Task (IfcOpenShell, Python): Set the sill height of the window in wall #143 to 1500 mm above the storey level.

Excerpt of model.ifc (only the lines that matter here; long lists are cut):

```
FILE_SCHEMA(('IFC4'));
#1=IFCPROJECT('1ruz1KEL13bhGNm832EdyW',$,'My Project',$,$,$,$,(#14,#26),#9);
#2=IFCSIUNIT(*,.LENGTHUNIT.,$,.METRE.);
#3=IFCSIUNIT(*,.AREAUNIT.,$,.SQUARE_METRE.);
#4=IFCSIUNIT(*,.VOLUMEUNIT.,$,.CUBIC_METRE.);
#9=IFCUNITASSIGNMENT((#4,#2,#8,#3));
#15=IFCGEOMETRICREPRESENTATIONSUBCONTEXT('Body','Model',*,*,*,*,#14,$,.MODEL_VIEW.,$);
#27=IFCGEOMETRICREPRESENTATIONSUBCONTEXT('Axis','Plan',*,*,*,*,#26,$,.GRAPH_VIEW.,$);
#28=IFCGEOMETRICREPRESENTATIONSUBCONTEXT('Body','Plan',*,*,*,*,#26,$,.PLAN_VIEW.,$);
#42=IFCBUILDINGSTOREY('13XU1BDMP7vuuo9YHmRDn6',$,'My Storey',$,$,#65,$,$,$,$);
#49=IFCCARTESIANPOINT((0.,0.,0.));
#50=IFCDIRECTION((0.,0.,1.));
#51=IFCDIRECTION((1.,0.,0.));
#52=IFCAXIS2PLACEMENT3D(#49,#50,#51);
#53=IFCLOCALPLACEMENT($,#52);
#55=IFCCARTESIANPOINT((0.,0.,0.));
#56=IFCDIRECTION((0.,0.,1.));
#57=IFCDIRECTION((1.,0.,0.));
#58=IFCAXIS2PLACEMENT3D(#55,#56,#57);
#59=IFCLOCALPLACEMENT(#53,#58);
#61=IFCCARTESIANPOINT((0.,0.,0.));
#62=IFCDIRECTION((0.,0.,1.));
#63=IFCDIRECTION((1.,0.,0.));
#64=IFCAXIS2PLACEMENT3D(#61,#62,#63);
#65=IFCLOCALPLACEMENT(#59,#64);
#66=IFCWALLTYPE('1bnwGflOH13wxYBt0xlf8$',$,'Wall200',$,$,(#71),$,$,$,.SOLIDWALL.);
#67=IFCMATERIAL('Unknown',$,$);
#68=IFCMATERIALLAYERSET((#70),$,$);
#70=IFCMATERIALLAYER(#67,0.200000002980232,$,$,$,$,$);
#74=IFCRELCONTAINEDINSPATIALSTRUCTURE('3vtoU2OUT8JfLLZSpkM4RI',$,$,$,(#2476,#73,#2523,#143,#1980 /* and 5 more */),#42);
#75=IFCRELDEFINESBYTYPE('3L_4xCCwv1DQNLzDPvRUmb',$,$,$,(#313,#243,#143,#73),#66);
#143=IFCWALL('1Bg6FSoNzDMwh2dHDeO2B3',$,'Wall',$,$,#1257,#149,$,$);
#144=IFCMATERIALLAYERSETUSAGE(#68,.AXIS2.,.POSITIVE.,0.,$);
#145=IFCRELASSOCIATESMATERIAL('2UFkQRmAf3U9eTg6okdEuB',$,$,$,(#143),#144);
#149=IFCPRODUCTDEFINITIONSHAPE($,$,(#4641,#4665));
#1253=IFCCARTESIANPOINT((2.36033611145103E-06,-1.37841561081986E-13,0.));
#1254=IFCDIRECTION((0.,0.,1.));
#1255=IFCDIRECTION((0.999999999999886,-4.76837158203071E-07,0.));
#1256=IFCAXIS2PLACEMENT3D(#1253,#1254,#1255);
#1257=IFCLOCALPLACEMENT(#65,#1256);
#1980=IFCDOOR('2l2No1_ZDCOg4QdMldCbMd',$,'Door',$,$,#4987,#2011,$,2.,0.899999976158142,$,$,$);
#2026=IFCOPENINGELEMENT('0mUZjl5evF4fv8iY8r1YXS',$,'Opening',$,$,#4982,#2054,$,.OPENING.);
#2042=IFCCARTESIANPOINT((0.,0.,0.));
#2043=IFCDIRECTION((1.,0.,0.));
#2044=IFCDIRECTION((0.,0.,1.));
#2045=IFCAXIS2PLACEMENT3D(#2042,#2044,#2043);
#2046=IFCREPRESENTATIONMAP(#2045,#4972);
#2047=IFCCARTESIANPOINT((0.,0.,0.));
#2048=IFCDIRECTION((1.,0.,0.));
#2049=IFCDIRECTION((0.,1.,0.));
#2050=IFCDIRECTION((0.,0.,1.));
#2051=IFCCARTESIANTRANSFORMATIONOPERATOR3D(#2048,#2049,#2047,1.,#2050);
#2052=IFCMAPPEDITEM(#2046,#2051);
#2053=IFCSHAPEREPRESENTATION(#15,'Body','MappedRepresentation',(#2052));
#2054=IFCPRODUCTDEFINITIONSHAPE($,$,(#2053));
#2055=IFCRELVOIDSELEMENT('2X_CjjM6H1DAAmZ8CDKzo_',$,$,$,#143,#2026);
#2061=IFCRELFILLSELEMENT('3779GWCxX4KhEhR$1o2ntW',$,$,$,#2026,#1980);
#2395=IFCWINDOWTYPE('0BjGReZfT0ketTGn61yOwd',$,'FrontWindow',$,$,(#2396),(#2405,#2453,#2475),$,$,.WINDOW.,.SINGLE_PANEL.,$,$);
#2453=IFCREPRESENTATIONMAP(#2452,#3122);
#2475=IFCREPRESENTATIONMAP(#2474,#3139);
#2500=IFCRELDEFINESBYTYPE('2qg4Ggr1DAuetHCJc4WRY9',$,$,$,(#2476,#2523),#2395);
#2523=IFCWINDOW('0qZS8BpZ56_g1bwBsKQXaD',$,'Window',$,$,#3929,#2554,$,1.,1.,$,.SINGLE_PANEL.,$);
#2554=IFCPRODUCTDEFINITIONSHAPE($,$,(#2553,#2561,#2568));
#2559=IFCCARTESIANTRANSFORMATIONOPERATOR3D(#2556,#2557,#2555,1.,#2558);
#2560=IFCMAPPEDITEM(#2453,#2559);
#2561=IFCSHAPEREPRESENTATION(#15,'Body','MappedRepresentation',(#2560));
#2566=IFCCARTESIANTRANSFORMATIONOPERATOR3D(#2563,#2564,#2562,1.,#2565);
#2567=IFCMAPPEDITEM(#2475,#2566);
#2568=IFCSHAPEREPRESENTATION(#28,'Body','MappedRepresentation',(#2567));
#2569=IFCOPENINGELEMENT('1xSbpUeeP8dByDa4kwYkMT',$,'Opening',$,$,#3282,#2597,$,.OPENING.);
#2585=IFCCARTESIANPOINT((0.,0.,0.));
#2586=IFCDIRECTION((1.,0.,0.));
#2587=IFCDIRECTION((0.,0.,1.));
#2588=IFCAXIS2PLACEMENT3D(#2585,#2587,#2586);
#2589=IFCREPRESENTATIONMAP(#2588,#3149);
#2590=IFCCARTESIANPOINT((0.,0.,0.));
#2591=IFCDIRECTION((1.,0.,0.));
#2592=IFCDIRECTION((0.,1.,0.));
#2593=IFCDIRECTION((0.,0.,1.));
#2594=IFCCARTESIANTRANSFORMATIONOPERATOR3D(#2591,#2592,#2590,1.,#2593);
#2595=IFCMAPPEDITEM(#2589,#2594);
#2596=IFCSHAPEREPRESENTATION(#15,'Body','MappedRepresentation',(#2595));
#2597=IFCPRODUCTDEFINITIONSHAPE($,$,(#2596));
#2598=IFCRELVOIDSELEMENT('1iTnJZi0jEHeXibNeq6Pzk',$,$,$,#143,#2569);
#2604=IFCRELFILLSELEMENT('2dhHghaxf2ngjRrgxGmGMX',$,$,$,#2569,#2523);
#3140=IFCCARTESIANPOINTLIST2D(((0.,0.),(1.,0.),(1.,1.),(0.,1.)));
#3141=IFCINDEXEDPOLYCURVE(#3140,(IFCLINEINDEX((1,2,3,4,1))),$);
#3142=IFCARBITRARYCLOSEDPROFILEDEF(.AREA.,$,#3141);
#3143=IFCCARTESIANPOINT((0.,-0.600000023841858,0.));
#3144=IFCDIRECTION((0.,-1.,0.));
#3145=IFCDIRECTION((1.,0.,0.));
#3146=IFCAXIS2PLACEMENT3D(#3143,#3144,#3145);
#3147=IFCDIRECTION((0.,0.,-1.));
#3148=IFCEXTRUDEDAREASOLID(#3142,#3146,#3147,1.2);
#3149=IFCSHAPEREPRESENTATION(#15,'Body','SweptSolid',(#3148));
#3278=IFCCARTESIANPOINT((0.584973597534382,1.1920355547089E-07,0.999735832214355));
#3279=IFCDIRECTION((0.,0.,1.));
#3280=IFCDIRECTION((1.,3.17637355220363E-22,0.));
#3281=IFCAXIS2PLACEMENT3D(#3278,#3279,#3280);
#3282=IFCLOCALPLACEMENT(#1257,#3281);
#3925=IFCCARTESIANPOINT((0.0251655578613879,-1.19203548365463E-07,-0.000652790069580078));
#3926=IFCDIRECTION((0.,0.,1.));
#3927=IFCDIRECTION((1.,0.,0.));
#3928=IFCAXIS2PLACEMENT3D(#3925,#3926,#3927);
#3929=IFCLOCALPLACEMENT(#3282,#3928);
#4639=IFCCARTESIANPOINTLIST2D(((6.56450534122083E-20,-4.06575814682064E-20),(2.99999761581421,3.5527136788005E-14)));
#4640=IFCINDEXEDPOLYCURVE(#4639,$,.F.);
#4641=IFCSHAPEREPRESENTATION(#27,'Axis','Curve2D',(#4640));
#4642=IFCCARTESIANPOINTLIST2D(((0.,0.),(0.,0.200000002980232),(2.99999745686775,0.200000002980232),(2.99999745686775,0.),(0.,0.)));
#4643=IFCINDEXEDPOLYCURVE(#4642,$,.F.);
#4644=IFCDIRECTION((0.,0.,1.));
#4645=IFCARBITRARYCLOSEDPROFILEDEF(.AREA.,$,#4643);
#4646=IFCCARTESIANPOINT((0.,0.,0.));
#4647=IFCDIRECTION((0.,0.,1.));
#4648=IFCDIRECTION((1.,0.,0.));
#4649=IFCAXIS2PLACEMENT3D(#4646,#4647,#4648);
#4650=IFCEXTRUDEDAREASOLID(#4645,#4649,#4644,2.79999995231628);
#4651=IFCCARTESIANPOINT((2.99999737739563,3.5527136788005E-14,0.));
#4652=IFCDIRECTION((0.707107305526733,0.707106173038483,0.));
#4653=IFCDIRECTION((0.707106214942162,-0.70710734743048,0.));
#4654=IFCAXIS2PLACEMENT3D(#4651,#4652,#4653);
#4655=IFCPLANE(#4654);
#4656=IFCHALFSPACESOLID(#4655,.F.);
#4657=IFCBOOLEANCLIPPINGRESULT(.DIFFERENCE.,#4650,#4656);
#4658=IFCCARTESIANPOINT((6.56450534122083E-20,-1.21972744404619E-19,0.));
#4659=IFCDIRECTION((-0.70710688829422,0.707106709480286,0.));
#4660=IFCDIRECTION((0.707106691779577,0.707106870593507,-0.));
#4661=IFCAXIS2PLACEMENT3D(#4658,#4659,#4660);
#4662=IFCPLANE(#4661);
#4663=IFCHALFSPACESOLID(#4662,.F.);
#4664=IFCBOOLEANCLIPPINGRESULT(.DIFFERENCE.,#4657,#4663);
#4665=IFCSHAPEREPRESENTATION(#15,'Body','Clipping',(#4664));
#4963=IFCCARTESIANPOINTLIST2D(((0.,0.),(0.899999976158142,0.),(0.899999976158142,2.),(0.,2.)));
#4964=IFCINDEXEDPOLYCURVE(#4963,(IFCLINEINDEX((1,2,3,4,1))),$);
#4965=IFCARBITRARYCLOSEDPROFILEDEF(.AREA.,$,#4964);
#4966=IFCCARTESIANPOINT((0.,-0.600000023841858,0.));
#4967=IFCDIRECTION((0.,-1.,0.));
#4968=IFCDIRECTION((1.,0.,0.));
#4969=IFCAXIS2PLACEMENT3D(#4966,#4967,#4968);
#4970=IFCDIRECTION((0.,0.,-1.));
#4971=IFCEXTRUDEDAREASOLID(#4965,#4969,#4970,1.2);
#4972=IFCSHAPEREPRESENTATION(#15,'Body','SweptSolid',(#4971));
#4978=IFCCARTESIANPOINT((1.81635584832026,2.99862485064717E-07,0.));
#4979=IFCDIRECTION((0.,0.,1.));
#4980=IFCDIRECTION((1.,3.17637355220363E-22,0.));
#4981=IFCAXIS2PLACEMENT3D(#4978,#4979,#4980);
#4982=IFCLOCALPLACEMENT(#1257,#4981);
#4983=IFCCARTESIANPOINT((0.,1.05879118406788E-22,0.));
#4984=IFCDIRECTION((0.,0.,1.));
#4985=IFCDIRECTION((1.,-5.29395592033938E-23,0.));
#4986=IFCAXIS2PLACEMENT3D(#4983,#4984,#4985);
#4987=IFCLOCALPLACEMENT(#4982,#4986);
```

```python
import numpy as np
import ifcopenshell
import ifcopenshell.api.geometry
import ifcopenshell.geom
import ifcopenshell.util.element
import ifcopenshell.util.placement
import ifcopenshell.util.shape
import ifcopenshell.util.unit

model = ifcopenshell.open("model.ifc")
unit_scale = ifcopenshell.util.unit.calculate_unit_scale(model)

window = model.by_id(2523)
opening = window.FillsVoids[0].RelatingOpeningElement
storey = ifcopenshell.util.element.get_container(window, ifc_class="IfcBuildingStorey")
level = ifcopenshell.util.placement.get_local_placement(storey.ObjectPlacement)[2, 3]

# The opening's origin need not be at the sill, so measure its lowest point.
shape = ifcopenshell.geom.create_shape(ifcopenshell.geom.settings(), opening)
bottom = ifcopenshell.util.shape.get_shape_bottom_elevation(shape, shape.geometry) / unit_scale
dz = level + 1.5 - bottom

shift = np.array([0.0, 0.0, dz])
# The window is placed relative to its opening, so it follows when the opening moves.
matrix = ifcopenshell.util.placement.get_local_placement(opening.ObjectPlacement)
matrix[:3, 3] += shift
ifcopenshell.api.geometry.edit_object_placement(
    model, product=opening, matrix=matrix, is_si=False, should_transform_children=True
)

print(f"moved by {dz * unit_scale:+.3f} m")

model.write("model_v2.ifc")
```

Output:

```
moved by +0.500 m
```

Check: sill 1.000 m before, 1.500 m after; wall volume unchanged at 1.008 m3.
